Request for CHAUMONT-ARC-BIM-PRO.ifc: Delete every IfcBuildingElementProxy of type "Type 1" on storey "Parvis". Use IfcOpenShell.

First a look at what the model holds.

```python
import ifcopenshell
import ifcopenshell.util.element

model = ifcopenshell.open("CHAUMONT-ARC-BIM-PRO.ifc")
print(model.schema)
storey = next(s for s in model.by_type("IfcBuildingStorey") if s.Name == "Parvis")
proxies = [e for e in ifcopenshell.util.element.get_decomposition(storey) if e.is_a("IfcBuildingElementProxy")]
seen = {}
for e in proxies:
    element_type = ifcopenshell.util.element.get_type(e)
    name = element_type.Name if element_type not in (None, e) else None
    seen[name] = seen.get(name, 0) + 1
for name, count in sorted(seen.items(), key=str):
    print(count, "x", name)
```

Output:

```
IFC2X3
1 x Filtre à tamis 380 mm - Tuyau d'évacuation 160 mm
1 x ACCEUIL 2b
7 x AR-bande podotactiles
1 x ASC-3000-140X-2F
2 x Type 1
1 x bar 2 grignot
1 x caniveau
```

```python
import ifcopenshell
import ifcopenshell.api.root
import ifcopenshell.util.element

model = ifcopenshell.open("CHAUMONT-ARC-BIM-PRO.ifc")

storey = next(s for s in model.by_type("IfcBuildingStorey") if s.Name == "Parvis")
proxies = [e for e in ifcopenshell.util.element.get_decomposition(storey) if e.is_a("IfcBuildingElementProxy")]
targets = [e for e in proxies if (t := ifcopenshell.util.element.get_type(e)) not in (None, e) and t.Name == "Type 1"]

for e in targets:
    ifcopenshell.api.root.remove_product(model, product=e)
print(len(targets), "removed")

model.write("CHAUMONT-ARC-BIM-PRO_edited.ifc")
```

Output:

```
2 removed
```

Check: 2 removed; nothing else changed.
